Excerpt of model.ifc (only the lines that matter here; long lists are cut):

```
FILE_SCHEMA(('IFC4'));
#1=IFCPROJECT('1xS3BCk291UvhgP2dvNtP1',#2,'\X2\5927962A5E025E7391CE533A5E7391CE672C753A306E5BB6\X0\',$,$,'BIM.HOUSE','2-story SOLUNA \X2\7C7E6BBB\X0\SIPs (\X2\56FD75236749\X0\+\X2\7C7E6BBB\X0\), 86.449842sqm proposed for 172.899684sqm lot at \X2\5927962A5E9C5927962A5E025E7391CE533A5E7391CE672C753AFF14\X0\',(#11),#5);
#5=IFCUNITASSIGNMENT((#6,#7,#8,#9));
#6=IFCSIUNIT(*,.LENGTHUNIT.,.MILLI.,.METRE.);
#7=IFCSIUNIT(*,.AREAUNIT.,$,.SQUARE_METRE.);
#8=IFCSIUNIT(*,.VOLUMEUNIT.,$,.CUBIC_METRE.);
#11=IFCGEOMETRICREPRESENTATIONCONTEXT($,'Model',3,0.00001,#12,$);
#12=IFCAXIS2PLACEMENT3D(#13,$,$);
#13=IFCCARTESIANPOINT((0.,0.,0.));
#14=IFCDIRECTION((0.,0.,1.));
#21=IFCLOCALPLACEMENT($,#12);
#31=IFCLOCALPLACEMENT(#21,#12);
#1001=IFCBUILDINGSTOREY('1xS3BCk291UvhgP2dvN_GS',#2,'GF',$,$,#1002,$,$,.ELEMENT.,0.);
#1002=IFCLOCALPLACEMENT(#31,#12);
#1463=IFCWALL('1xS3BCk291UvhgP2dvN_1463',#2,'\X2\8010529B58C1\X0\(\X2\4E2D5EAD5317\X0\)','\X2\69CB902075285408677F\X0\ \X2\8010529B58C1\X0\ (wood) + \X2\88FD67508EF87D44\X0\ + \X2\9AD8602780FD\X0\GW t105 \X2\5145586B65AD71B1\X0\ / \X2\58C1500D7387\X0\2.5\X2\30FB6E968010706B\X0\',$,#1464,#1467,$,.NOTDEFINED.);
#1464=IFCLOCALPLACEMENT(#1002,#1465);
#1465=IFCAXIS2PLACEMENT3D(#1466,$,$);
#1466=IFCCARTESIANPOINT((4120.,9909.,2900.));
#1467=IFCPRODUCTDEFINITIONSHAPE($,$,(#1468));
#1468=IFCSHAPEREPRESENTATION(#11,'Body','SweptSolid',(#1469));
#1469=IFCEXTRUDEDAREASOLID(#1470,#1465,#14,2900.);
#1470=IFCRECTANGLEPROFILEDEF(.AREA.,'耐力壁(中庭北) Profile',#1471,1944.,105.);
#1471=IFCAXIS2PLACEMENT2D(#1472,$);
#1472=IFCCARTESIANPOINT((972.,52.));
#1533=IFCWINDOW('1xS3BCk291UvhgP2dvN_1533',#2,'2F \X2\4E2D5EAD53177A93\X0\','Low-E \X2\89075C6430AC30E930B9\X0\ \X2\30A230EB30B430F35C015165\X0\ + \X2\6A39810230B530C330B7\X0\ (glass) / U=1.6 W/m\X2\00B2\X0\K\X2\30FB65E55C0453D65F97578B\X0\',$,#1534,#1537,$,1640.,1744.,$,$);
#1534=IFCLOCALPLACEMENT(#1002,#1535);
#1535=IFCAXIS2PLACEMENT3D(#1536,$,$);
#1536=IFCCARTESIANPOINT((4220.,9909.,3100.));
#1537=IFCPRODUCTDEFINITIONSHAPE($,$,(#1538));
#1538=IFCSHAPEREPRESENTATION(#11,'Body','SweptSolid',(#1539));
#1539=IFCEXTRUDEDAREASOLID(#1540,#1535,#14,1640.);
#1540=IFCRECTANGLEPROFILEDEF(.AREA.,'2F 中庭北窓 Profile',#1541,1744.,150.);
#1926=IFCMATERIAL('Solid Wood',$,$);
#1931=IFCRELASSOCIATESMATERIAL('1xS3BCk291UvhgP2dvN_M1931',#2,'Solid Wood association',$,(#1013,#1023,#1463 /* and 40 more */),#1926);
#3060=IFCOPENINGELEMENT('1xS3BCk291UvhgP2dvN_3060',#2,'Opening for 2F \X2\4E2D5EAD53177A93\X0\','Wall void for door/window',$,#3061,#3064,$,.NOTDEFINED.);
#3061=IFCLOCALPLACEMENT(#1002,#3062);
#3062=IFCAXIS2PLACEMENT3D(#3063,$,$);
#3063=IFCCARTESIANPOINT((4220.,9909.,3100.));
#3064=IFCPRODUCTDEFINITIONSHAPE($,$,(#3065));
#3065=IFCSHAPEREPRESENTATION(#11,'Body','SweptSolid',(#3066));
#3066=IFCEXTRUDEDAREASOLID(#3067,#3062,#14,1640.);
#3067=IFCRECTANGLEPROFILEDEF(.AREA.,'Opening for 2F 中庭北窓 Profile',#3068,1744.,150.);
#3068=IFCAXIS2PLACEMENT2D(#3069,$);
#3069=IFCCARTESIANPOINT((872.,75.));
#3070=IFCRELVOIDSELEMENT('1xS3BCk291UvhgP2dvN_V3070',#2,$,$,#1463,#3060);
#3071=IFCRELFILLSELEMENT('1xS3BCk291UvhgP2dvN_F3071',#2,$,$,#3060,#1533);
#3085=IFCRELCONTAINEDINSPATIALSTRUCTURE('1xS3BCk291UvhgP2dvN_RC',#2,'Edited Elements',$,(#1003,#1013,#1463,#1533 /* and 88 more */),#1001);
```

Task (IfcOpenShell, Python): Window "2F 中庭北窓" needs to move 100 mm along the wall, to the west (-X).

```python
import ifcopenshell
import ifcopenshell.api.geometry
import ifcopenshell.util.placement
import ifcopenshell.util.unit

model = ifcopenshell.open("model.ifc")
unit_scale = ifcopenshell.util.unit.calculate_unit_scale(model)

window = model.by_id(1533)
opening = window.FillsVoids[0].RelatingOpeningElement
wall = opening.VoidsElements[0].RelatingBuildingElement

wall_matrix = ifcopenshell.util.placement.get_local_placement(wall.ObjectPlacement)
shift = wall_matrix[:3, 0] * -0.1 / unit_scale
before = ifcopenshell.util.placement.get_local_placement(window.ObjectPlacement)[:3, 3].copy()

# The window is not placed relative to its opening, so move both.
for product in (opening, window):
    matrix = ifcopenshell.util.placement.get_local_placement(product.ObjectPlacement)
    matrix[:3, 3] += shift
    ifcopenshell.api.geometry.edit_object_placement(model, product=product, matrix=matrix, is_si=False)

after = ifcopenshell.util.placement.get_local_placement(window.ObjectPlacement)[:3, 3]
print("window moved by", (after - before).round(3) + 0.0)

model.write("model_edited.ifc")
```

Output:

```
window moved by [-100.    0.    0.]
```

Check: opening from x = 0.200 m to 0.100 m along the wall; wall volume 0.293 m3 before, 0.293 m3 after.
